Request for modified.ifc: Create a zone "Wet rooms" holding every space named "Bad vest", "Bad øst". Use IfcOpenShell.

First a look at what the model holds.

```python
import ifcopenshell

model = ifcopenshell.open("modified.ifc")
print(model.schema)
seen = {}
for space in model.by_type("IfcSpace"):
    seen[space.LongName] = seen.get(space.LongName, 0) + 1
for name, count in sorted(seen.items(), key=str):
    print(count, "x", name)
print("zones:", [z.Name for z in model.by_type("IfcZone")][:20])
```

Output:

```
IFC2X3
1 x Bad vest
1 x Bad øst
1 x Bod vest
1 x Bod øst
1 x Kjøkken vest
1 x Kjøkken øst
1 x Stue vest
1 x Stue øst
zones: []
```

```python
import ifcopenshell
import ifcopenshell.api.group
import ifcopenshell.api.root

model = ifcopenshell.open("modified.ifc")

names = {"Bad vest", "Bad øst"}
spaces = [s for s in model.by_type("IfcSpace") if s.LongName in names]

zone = ifcopenshell.api.root.create_entity(model, ifc_class="IfcZone", name="Wet rooms")
ifcopenshell.api.group.assign_group(model, products=spaces, group=zone)
print(len(spaces), "spaces in", zone.Name)

model.write("modified_updated.ifc")
```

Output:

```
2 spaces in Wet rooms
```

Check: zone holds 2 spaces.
